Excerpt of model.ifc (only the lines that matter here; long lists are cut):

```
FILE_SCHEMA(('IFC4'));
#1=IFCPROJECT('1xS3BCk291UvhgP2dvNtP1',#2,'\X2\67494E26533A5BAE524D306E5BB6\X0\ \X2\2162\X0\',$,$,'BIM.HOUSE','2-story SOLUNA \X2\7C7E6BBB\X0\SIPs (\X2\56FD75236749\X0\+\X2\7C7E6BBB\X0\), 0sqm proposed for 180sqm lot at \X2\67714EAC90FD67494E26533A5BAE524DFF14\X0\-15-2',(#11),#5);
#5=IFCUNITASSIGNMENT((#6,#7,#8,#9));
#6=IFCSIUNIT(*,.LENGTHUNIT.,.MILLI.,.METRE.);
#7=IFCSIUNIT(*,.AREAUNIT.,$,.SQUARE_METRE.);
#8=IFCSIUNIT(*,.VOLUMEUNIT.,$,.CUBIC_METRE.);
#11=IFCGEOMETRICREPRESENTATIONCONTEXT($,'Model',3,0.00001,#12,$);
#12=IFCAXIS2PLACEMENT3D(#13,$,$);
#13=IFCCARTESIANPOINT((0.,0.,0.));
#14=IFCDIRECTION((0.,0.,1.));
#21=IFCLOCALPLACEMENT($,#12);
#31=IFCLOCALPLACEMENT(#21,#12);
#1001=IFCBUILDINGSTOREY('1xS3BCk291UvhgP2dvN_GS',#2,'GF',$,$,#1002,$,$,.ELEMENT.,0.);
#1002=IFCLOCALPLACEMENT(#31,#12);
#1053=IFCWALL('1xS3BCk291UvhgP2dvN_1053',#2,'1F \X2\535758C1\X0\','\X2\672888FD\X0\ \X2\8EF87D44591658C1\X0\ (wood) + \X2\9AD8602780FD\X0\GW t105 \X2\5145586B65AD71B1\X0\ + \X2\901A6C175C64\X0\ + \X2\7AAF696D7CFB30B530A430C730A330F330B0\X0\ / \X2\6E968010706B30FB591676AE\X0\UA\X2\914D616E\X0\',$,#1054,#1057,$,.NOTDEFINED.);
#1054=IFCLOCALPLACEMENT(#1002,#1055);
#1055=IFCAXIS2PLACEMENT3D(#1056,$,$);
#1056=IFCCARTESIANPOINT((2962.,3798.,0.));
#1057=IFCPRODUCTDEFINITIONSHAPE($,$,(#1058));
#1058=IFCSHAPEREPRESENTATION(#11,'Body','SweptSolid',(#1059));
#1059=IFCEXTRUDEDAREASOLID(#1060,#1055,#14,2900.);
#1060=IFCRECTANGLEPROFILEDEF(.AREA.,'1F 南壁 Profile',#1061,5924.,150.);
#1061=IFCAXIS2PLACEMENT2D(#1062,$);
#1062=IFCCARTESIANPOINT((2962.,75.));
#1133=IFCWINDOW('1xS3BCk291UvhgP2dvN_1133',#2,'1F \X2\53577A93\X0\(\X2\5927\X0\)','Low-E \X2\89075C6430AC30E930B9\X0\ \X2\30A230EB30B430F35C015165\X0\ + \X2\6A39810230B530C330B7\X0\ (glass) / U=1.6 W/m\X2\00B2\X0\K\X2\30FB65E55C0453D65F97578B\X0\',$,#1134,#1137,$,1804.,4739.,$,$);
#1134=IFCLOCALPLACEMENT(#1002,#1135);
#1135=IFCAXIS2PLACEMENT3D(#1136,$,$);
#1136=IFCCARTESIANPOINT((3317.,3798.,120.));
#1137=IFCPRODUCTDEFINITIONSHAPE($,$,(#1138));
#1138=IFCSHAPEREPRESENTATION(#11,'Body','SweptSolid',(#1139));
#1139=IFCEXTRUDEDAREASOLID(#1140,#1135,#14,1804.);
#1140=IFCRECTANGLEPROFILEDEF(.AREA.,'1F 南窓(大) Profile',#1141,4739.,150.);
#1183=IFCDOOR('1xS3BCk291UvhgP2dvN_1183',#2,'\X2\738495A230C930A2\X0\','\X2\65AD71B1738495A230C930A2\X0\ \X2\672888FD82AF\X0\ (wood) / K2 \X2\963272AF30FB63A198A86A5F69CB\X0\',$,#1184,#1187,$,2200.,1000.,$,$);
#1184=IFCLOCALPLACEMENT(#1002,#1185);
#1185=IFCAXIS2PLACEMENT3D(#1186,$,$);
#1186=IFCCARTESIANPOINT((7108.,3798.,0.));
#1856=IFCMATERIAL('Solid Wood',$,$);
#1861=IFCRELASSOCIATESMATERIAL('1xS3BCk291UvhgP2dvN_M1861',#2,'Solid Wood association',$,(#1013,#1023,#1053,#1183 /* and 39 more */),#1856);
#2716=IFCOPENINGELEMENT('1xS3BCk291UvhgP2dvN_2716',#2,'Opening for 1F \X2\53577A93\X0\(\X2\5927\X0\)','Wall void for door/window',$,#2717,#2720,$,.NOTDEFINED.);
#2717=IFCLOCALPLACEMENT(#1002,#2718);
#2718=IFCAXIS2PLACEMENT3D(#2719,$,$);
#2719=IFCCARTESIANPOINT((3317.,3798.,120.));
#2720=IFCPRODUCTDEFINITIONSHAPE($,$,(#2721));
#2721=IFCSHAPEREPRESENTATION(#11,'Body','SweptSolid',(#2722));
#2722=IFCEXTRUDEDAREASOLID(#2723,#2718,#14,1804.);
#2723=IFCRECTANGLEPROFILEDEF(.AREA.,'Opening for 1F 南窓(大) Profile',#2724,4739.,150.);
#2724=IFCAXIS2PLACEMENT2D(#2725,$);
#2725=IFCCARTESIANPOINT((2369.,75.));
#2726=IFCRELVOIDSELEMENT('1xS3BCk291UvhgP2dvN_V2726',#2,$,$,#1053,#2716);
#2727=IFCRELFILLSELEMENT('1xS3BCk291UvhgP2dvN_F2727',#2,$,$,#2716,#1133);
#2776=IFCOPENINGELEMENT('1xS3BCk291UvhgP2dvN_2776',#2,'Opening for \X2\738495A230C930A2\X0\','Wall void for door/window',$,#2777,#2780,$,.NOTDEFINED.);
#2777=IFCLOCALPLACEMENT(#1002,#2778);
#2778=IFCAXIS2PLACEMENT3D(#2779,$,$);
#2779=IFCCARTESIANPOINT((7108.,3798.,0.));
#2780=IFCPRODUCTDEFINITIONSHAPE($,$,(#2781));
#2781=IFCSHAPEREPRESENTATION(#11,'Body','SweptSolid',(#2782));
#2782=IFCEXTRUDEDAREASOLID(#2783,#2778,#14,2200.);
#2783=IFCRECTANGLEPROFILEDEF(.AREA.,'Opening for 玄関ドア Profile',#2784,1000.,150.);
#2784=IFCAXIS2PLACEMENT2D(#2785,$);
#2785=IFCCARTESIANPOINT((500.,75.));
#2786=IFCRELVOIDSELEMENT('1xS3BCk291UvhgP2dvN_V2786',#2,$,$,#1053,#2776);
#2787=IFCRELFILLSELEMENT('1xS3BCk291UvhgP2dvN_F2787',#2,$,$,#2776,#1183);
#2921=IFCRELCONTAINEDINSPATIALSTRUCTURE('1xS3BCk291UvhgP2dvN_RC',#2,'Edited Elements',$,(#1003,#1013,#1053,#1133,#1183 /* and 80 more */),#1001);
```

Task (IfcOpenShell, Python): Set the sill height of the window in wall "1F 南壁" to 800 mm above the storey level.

```python
import numpy as np
import ifcopenshell
import ifcopenshell.api.geometry
import ifcopenshell.geom
import ifcopenshell.util.element
import ifcopenshell.util.placement
import ifcopenshell.util.shape
import ifcopenshell.util.unit

model = ifcopenshell.open("model.ifc")
unit_scale = ifcopenshell.util.unit.calculate_unit_scale(model)

window = model.by_guid("1xS3BCk291UvhgP2dvN_1133")
opening = window.FillsVoids[0].RelatingOpeningElement
storey = ifcopenshell.util.element.get_container(window, ifc_class="IfcBuildingStorey")
level = ifcopenshell.util.placement.get_local_placement(storey.ObjectPlacement)[2, 3]

# The opening's origin need not be at the sill, so measure its lowest point.
shape = ifcopenshell.geom.create_shape(ifcopenshell.geom.settings(), opening)
bottom = ifcopenshell.util.shape.get_shape_bottom_elevation(shape, shape.geometry) / unit_scale
dz = level + 800.0 - bottom

shift = np.array([0.0, 0.0, dz])
# The window is not placed relative to its opening, so move both.
for product in (opening, window):
    matrix = ifcopenshell.util.placement.get_local_placement(product.ObjectPlacement)
    matrix[:3, 3] += shift
    ifcopenshell.api.geometry.edit_object_placement(model, product=product, matrix=matrix, is_si=False)

print(f"moved by {dz * unit_scale:+.3f} m")

model.write("model-out.ifc")
```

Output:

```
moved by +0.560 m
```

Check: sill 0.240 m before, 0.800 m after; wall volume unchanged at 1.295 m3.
